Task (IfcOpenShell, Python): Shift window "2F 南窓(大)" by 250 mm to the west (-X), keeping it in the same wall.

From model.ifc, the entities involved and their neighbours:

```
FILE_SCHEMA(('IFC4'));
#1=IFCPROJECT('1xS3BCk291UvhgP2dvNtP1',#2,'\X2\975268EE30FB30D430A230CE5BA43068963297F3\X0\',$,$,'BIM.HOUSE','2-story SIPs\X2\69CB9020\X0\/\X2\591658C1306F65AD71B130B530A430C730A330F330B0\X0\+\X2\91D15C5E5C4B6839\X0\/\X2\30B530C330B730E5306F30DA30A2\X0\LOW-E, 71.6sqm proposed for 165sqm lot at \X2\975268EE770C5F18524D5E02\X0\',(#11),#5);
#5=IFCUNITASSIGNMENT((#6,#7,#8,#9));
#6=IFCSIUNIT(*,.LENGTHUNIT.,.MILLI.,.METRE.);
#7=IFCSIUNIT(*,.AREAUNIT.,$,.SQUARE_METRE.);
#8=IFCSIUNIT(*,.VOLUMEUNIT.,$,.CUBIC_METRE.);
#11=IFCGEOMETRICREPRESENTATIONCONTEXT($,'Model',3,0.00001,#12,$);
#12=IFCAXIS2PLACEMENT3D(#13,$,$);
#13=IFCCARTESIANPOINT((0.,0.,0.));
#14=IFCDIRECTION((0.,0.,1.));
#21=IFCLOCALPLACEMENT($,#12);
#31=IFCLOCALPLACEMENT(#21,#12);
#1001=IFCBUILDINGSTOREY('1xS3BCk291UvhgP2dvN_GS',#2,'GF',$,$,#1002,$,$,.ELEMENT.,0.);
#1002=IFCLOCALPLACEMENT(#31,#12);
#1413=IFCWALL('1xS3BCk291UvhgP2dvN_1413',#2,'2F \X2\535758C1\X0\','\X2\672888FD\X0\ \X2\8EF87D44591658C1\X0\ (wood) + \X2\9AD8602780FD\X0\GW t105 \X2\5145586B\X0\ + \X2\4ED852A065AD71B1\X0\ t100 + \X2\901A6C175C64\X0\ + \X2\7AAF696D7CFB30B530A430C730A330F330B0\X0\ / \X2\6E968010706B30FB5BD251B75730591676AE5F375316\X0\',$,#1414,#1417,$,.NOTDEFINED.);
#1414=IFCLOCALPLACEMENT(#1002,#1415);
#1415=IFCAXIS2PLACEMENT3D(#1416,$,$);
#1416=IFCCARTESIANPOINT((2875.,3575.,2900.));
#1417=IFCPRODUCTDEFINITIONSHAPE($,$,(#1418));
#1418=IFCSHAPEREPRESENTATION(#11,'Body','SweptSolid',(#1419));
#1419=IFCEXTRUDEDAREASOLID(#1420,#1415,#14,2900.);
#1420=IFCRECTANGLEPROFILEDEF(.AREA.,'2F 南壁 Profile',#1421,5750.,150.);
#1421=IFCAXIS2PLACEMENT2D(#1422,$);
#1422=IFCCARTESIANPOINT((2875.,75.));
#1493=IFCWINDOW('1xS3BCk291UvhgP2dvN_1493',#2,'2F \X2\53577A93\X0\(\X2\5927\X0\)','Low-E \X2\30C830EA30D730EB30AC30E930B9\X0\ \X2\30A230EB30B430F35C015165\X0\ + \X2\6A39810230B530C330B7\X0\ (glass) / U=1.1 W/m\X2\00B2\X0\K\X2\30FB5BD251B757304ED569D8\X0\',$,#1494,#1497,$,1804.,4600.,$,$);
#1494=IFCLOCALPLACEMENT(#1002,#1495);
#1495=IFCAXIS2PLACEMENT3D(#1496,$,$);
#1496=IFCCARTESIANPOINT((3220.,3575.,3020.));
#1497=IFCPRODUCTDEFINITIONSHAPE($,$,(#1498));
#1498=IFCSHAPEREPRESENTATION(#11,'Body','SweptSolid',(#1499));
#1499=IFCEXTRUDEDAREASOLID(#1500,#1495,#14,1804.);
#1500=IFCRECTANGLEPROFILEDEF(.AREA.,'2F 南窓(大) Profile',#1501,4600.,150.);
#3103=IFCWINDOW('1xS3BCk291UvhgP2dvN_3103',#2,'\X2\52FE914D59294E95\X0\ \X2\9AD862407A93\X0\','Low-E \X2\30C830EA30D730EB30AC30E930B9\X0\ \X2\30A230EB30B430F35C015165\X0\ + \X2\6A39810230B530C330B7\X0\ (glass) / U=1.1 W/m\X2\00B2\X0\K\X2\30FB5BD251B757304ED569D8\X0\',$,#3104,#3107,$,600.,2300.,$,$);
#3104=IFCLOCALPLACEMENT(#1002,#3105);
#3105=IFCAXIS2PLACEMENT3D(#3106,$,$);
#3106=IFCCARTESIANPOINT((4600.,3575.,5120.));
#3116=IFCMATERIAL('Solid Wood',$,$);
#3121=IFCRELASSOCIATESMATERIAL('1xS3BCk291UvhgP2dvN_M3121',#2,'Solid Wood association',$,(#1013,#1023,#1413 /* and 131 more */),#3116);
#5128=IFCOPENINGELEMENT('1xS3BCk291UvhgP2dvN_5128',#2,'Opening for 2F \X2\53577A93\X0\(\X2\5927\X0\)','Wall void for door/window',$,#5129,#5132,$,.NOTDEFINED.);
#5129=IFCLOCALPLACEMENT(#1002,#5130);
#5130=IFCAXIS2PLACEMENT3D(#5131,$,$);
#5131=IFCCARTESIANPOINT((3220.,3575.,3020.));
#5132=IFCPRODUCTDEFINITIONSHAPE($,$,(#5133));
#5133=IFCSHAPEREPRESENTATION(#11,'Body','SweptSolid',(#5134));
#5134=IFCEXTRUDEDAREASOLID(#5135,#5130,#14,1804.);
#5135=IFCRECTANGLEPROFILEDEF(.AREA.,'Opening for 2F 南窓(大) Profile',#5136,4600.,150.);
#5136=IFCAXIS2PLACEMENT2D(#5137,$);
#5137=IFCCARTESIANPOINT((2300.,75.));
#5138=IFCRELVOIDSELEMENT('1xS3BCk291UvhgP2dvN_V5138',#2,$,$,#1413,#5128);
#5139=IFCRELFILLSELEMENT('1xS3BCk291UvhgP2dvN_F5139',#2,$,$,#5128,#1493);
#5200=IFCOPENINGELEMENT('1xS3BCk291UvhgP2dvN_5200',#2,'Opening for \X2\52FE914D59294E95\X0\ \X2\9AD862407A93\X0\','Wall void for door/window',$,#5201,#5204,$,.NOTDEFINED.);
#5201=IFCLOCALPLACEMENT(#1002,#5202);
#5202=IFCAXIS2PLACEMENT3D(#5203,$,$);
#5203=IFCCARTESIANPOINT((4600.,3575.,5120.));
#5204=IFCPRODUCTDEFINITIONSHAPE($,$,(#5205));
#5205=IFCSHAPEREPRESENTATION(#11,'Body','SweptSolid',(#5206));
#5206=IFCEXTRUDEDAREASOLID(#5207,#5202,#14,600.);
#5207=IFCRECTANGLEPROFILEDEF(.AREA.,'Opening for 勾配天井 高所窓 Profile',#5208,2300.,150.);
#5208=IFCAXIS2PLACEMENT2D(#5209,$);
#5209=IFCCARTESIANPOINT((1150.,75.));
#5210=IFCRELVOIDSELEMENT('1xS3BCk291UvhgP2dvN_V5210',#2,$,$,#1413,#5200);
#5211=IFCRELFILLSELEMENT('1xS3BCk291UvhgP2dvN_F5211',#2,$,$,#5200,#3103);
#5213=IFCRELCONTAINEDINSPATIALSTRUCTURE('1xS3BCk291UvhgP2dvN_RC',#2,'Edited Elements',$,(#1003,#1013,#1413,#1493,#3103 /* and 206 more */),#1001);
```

```python
import ifcopenshell
import ifcopenshell.api.geometry
import ifcopenshell.util.placement
import ifcopenshell.util.unit

model = ifcopenshell.open("model.ifc")
unit_scale = ifcopenshell.util.unit.calculate_unit_scale(model)

window = model.by_guid("1xS3BCk291UvhgP2dvN_1493")
opening = window.FillsVoids[0].RelatingOpeningElement
wall = opening.VoidsElements[0].RelatingBuildingElement

wall_matrix = ifcopenshell.util.placement.get_local_placement(wall.ObjectPlacement)
shift = wall_matrix[:3, 0] * -0.25 / unit_scale
before = ifcopenshell.util.placement.get_local_placement(window.ObjectPlacement)[:3, 3].copy()

# The window is not placed relative to its opening, so move both.
for product in (opening, window):
    matrix = ifcopenshell.util.placement.get_local_placement(product.ObjectPlacement)
    matrix[:3, 3] += shift
    ifcopenshell.api.geometry.edit_object_placement(model, product=product, matrix=matrix, is_si=False)

after = ifcopenshell.util.placement.get_local_placement(window.ObjectPlacement)[:3, 3]
print("window moved by", (after - before).round(3) + 0.0)

model.write("model_updated.ifc")
```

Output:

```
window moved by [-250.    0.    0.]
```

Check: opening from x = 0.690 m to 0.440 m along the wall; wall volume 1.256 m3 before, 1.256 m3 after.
